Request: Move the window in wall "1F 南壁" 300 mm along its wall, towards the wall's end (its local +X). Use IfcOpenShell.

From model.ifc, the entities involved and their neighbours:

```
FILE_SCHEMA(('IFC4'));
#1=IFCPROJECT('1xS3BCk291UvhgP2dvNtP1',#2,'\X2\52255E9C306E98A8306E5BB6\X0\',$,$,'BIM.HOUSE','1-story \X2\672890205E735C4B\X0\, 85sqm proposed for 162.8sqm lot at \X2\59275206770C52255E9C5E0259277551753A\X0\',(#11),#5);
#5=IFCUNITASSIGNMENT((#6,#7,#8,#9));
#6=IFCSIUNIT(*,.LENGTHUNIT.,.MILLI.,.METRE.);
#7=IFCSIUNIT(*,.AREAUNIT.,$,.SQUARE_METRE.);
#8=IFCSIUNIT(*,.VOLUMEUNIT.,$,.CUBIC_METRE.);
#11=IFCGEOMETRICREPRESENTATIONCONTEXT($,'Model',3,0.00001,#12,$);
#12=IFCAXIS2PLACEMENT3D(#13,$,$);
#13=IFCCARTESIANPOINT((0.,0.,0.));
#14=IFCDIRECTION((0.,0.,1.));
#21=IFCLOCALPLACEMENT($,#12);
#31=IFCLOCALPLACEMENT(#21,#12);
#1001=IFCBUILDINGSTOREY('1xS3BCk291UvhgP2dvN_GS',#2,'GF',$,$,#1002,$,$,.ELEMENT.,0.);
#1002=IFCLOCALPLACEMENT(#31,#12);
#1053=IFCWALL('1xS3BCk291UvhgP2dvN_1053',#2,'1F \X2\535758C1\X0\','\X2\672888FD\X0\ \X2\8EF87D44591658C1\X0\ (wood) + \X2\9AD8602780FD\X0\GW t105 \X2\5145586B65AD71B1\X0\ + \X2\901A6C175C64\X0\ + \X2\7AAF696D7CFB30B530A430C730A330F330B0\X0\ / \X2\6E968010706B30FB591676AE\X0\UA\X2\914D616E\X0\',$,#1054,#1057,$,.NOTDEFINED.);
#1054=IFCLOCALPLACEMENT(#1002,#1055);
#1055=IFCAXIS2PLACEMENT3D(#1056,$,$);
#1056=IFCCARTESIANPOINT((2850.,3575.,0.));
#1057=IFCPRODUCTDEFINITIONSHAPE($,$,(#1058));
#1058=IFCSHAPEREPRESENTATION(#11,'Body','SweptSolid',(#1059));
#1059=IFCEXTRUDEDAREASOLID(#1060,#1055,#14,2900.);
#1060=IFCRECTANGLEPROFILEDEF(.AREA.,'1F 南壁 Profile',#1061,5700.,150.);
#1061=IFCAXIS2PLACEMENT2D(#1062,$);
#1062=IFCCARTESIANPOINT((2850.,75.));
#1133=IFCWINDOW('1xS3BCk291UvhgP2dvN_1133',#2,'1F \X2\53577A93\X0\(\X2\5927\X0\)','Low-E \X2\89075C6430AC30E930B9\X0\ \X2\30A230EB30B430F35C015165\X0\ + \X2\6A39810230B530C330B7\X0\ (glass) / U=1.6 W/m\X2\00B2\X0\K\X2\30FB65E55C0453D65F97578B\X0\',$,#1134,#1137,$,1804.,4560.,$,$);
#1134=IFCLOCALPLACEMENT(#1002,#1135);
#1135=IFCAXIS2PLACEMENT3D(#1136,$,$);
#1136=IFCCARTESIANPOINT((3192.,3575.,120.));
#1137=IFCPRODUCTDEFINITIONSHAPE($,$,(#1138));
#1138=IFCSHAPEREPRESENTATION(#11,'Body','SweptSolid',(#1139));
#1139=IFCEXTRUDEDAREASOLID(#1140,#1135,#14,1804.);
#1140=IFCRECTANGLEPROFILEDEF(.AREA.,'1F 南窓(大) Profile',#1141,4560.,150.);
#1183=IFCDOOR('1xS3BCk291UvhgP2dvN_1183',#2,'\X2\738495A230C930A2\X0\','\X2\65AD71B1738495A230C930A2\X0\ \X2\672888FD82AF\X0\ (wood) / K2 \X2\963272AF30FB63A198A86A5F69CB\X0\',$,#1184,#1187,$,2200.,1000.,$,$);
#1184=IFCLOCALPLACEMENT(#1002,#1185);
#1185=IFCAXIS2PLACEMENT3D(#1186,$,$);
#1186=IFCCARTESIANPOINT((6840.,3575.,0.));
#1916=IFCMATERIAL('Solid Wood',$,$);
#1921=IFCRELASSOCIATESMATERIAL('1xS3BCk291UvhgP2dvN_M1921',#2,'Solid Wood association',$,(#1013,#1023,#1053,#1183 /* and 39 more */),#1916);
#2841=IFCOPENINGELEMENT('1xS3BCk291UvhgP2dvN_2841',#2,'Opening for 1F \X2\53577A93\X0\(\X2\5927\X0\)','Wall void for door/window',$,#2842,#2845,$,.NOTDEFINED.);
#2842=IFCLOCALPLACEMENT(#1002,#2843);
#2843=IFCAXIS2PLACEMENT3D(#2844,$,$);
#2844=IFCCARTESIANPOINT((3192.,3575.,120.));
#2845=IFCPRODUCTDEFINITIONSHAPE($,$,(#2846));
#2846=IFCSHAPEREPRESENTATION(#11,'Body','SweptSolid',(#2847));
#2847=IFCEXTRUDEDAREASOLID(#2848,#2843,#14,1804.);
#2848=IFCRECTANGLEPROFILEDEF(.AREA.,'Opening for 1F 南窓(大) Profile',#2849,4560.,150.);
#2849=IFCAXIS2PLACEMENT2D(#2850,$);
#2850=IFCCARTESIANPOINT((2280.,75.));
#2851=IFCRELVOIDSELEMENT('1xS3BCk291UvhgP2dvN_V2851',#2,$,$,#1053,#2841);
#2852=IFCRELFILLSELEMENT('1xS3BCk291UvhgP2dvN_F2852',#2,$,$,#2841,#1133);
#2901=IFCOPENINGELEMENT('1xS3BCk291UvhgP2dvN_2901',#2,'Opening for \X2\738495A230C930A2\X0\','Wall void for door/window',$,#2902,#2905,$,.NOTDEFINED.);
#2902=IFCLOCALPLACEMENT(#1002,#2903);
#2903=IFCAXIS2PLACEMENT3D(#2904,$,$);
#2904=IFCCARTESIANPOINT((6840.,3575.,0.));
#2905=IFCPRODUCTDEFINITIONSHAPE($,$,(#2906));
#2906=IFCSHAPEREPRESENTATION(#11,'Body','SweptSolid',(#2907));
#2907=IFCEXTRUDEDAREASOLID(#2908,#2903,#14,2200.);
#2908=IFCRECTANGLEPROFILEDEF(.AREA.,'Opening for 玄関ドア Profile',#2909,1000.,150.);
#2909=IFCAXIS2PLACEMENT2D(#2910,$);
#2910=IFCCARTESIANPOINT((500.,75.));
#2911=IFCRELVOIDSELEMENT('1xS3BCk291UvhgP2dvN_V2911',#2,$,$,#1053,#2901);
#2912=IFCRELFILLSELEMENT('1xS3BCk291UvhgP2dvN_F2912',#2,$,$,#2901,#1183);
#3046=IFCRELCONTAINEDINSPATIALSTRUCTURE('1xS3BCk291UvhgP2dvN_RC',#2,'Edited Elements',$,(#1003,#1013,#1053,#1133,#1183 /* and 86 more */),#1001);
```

```python
import ifcopenshell
import ifcopenshell.api.geometry
import ifcopenshell.util.placement
import ifcopenshell.util.unit

model = ifcopenshell.open("model.ifc")
unit_scale = ifcopenshell.util.unit.calculate_unit_scale(model)

window = model.by_guid("1xS3BCk291UvhgP2dvN_1133")
opening = window.FillsVoids[0].RelatingOpeningElement
wall = opening.VoidsElements[0].RelatingBuildingElement

wall_matrix = ifcopenshell.util.placement.get_local_placement(wall.ObjectPlacement)
shift = wall_matrix[:3, 0] * 0.3 / unit_scale
before = ifcopenshell.util.placement.get_local_placement(window.ObjectPlacement)[:3, 3].copy()

# The window is not placed relative to its opening, so move both.
for product in (opening, window):
    matrix = ifcopenshell.util.placement.get_local_placement(product.ObjectPlacement)
    matrix[:3, 3] += shift
    ifcopenshell.api.geometry.edit_object_placement(model, product=product, matrix=matrix, is_si=False)

after = ifcopenshell.util.placement.get_local_placement(window.ObjectPlacement)[:3, 3]
print("window moved by", (after - before).round(3) + 0.0)

model.write("model_rev.ifc")
```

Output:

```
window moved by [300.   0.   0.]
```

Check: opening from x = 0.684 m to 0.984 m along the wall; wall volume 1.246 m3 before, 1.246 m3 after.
